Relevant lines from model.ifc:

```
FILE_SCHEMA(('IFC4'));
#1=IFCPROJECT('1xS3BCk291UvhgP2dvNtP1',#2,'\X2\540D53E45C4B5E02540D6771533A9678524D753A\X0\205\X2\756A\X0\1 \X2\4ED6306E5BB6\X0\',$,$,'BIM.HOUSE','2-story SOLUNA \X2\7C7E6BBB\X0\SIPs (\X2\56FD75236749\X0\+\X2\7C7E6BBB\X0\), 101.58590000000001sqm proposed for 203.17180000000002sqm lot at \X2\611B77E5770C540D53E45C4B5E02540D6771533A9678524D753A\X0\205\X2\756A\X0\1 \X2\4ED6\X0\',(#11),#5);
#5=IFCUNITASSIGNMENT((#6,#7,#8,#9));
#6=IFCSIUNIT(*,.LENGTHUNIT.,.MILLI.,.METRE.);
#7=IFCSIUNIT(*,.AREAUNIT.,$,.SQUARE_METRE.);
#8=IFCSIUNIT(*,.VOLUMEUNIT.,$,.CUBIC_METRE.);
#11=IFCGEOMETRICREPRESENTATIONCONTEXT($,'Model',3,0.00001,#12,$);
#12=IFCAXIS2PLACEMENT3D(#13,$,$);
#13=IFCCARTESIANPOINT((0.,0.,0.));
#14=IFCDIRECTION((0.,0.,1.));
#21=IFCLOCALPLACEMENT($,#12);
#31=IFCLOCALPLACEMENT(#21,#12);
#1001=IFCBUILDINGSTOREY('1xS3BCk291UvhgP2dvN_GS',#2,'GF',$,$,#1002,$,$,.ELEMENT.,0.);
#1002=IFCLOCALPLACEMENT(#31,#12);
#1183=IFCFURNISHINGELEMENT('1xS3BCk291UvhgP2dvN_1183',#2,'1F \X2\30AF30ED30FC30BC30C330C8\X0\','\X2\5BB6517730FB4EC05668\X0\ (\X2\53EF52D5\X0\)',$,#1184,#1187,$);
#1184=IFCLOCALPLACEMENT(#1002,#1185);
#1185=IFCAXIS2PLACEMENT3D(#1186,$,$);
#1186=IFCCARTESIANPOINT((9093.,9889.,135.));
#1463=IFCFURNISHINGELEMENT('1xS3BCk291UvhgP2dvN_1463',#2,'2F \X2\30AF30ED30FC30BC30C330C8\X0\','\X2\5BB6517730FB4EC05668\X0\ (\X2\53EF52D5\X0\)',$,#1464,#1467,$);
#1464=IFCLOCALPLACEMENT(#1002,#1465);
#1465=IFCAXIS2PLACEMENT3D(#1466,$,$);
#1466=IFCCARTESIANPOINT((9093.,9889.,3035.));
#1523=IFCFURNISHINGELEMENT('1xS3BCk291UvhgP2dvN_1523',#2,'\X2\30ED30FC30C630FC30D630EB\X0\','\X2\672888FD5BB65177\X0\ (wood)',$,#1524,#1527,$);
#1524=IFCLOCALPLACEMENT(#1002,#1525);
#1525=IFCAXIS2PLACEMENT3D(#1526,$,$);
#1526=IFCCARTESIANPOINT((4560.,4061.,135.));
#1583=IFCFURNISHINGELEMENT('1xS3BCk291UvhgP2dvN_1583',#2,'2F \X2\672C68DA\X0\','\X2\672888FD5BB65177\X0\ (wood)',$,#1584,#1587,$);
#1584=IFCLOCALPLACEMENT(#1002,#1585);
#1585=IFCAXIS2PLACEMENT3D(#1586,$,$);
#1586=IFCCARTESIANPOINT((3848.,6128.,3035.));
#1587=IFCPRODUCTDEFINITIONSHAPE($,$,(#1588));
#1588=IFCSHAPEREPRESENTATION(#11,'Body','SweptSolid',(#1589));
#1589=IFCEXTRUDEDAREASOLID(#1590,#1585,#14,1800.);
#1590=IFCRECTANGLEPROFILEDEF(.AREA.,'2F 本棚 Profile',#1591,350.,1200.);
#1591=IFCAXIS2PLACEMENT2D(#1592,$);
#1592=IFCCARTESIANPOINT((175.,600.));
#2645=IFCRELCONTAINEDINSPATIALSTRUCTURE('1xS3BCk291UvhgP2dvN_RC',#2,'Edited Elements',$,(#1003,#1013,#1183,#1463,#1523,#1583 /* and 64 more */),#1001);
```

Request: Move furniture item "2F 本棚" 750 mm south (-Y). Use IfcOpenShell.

```python
import ifcopenshell
import ifcopenshell.api.geometry
import ifcopenshell.util.placement

model = ifcopenshell.open("model.ifc")

item = model.by_guid("1xS3BCk291UvhgP2dvN_1583")
matrix = ifcopenshell.util.placement.get_local_placement(item.ObjectPlacement)
matrix[1, 3] -= 750.0
ifcopenshell.api.geometry.edit_object_placement(model, product=item, matrix=matrix, is_si=False)

print(ifcopenshell.util.placement.get_local_placement(item.ObjectPlacement).round(3) + 0.0)

model.write("model_v2.ifc")
```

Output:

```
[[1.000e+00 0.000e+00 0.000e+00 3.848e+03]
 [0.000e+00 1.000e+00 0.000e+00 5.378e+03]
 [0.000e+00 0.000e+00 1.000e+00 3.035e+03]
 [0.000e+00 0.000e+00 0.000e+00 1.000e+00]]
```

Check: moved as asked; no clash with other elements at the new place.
